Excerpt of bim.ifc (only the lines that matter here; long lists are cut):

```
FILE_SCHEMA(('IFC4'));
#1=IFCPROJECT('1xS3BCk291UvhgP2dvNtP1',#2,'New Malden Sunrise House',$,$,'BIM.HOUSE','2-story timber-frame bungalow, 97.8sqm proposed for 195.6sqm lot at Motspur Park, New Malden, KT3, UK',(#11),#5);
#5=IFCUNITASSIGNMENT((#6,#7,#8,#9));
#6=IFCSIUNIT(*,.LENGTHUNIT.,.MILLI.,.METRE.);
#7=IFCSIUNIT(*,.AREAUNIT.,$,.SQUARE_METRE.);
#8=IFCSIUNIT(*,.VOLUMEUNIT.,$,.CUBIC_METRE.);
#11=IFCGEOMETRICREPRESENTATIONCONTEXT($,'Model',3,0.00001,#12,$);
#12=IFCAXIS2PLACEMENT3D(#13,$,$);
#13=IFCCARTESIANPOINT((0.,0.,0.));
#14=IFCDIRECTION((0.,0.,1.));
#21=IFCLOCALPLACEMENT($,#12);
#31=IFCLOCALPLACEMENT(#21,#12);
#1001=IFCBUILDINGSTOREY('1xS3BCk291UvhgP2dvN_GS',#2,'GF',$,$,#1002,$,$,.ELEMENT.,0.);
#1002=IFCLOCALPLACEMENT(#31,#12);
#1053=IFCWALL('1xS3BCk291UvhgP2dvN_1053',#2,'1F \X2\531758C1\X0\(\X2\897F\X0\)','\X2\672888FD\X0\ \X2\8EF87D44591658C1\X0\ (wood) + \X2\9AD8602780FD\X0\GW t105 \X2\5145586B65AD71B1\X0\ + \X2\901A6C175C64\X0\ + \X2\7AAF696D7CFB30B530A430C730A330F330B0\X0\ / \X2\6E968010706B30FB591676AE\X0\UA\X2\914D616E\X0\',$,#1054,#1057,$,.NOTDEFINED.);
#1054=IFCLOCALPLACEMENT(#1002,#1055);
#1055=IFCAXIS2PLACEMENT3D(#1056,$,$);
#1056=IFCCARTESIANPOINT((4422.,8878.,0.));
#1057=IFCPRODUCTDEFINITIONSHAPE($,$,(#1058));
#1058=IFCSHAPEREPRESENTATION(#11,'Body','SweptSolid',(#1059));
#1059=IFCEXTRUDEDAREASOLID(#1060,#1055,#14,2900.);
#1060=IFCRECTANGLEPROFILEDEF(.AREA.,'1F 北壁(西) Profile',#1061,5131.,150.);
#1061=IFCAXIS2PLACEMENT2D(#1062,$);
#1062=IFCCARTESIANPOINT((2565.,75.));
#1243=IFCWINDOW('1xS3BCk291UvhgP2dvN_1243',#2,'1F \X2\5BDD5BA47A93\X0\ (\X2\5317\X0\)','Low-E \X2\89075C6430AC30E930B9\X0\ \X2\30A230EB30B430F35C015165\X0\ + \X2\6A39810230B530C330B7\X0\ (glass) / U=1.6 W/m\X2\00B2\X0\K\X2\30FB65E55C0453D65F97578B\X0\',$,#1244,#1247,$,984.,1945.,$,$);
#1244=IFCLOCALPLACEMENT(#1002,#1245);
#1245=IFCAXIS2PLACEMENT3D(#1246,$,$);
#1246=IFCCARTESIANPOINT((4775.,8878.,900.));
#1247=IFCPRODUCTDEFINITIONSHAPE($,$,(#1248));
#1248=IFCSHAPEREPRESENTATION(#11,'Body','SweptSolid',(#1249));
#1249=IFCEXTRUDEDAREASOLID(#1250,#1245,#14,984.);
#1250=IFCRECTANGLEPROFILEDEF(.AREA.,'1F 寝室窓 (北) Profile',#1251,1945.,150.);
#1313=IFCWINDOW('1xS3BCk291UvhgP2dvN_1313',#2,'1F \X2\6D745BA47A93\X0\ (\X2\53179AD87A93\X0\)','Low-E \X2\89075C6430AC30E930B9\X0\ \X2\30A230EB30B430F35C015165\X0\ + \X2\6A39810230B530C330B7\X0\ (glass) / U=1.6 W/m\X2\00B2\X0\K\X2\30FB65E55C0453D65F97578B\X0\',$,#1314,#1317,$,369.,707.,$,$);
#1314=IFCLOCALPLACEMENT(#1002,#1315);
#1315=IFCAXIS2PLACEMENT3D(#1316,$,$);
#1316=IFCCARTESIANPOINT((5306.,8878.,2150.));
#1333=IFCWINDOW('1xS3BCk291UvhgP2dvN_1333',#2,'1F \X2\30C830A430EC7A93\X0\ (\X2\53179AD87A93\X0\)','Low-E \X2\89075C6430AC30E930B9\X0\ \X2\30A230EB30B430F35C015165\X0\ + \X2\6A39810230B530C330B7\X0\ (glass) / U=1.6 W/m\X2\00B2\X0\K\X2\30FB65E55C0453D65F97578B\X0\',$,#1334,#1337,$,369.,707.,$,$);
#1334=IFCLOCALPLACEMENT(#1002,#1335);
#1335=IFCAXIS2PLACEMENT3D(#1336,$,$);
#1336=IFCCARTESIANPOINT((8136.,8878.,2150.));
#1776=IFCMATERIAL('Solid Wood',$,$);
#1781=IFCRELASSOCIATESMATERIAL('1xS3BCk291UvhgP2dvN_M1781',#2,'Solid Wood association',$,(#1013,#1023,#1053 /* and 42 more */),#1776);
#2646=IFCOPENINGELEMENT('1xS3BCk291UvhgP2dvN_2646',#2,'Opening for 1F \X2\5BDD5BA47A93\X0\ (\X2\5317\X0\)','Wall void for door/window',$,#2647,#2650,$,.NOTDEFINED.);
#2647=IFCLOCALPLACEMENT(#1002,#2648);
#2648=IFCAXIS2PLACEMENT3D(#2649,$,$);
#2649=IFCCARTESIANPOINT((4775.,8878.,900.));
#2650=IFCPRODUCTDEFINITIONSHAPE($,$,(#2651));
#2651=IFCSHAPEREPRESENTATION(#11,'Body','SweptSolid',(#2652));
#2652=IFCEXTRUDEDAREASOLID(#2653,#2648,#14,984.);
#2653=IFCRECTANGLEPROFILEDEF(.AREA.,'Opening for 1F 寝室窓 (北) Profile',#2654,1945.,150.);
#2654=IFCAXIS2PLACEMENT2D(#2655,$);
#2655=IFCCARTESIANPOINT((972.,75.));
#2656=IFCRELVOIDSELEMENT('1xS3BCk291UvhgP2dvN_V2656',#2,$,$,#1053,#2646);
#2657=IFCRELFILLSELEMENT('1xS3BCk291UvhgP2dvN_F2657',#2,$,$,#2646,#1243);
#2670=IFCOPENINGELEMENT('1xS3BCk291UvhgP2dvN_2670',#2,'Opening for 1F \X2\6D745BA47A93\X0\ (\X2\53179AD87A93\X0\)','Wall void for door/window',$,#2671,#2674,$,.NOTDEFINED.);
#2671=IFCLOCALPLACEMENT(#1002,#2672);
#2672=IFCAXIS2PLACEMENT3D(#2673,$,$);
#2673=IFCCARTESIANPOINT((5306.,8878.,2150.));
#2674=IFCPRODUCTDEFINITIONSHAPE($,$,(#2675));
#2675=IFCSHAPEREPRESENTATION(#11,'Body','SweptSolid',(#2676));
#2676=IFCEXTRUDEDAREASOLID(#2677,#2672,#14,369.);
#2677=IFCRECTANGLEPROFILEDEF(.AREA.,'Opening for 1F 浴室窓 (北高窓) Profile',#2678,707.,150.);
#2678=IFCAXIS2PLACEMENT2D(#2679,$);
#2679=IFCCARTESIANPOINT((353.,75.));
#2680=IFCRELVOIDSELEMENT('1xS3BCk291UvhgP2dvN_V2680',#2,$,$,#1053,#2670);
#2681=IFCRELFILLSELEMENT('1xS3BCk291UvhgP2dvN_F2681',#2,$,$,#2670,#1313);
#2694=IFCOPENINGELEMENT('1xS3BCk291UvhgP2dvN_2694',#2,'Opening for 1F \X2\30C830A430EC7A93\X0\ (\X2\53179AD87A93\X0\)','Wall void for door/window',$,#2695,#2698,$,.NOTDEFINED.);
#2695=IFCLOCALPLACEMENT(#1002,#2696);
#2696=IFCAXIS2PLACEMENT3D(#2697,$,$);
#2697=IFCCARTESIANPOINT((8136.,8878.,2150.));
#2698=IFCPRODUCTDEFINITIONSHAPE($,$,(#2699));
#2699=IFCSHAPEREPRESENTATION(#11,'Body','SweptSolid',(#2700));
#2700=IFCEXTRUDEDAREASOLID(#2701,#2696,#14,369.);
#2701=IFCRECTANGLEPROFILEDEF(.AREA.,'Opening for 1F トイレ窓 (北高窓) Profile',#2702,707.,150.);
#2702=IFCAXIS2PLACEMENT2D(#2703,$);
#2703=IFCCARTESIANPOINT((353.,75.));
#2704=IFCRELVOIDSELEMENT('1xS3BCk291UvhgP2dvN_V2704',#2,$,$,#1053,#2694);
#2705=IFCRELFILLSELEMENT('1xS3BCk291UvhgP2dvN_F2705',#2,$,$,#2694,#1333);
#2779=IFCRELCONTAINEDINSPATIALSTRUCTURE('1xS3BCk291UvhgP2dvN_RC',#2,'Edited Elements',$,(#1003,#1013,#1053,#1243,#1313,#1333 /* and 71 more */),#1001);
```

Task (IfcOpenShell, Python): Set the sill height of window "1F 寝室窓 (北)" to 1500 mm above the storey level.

```python
import numpy as np
import ifcopenshell
import ifcopenshell.api.geometry
import ifcopenshell.geom
import ifcopenshell.util.element
import ifcopenshell.util.placement
import ifcopenshell.util.shape
import ifcopenshell.util.unit

model = ifcopenshell.open("bim.ifc")
unit_scale = ifcopenshell.util.unit.calculate_unit_scale(model)

window = model.by_id(1243)
opening = window.FillsVoids[0].RelatingOpeningElement
storey = ifcopenshell.util.element.get_container(window, ifc_class="IfcBuildingStorey")
level = ifcopenshell.util.placement.get_local_placement(storey.ObjectPlacement)[2, 3]

# The opening's origin need not be at the sill, so measure its lowest point.
shape = ifcopenshell.geom.create_shape(ifcopenshell.geom.settings(), opening)
bottom = ifcopenshell.util.shape.get_shape_bottom_elevation(shape, shape.geometry) / unit_scale
dz = level + 1500.0 - bottom

shift = np.array([0.0, 0.0, dz])
# The window is not placed relative to its opening, so move both.
for product in (opening, window):
    matrix = ifcopenshell.util.placement.get_local_placement(product.ObjectPlacement)
    matrix[:3, 3] += shift
    ifcopenshell.api.geometry.edit_object_placement(model, product=product, matrix=matrix, is_si=False)

print(f"moved by {dz * unit_scale:+.3f} m")

model.write("bim_v2.ifc")
```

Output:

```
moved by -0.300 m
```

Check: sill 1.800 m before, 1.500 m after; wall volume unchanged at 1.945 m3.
